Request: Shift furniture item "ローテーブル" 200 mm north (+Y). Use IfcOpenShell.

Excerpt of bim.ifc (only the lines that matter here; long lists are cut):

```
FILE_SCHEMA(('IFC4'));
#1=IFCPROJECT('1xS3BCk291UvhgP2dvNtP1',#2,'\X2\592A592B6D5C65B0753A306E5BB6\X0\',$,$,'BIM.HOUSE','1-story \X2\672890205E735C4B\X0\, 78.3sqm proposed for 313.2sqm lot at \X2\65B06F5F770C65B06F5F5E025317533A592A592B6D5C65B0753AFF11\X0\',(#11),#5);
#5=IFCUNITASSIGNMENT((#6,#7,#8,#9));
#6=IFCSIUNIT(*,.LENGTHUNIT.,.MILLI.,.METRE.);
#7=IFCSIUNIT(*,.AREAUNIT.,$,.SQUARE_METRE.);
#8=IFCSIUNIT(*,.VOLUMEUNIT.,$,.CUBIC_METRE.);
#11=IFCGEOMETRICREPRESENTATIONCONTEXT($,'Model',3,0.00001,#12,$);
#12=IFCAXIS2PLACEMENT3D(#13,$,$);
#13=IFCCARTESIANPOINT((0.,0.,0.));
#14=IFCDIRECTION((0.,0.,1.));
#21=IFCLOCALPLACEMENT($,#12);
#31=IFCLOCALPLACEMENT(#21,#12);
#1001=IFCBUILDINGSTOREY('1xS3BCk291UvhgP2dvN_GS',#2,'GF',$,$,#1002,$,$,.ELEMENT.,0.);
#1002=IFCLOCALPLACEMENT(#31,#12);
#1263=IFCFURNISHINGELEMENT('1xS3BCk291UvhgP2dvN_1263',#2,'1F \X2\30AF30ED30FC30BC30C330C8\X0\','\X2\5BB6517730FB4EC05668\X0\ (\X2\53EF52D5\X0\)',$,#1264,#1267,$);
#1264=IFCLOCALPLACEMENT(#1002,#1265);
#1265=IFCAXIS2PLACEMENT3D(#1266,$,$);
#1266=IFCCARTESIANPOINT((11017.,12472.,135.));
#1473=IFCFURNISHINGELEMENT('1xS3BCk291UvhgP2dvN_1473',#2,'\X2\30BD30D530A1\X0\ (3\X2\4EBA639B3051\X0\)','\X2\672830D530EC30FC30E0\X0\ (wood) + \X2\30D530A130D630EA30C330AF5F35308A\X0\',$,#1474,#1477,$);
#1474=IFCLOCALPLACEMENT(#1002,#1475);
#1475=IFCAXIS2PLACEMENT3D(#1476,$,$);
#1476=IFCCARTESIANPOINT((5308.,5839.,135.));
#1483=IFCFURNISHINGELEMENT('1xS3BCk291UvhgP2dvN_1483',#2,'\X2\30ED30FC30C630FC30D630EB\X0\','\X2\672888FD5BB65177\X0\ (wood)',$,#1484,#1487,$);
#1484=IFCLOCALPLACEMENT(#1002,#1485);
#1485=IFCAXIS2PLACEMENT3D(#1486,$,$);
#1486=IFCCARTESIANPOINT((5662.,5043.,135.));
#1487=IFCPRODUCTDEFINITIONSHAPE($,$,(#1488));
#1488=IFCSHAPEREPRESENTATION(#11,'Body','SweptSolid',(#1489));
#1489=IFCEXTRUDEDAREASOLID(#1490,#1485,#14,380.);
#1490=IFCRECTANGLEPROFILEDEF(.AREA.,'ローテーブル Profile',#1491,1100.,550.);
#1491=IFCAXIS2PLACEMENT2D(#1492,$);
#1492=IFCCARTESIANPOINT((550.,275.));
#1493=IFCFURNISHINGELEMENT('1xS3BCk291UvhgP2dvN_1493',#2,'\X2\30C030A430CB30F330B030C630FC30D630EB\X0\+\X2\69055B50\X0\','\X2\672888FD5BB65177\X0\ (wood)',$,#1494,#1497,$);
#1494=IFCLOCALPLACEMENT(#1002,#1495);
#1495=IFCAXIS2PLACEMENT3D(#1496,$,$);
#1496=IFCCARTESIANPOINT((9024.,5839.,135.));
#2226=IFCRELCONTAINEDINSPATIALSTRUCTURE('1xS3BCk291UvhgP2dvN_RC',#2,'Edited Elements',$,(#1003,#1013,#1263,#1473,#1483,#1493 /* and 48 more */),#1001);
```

```python
import ifcopenshell
import ifcopenshell.api.geometry
import ifcopenshell.util.placement
import ifcopenshell.util.unit

model = ifcopenshell.open("bim.ifc")
unit_scale = ifcopenshell.util.unit.calculate_unit_scale(model)

item = model.by_guid("1xS3BCk291UvhgP2dvN_1483")
matrix = ifcopenshell.util.placement.get_local_placement(item.ObjectPlacement)
matrix[1, 3] += 0.2 / unit_scale
ifcopenshell.api.geometry.edit_object_placement(model, product=item, matrix=matrix, is_si=False)

print(ifcopenshell.util.placement.get_local_placement(item.ObjectPlacement).round(3) + 0.0)

model.write("bim_edited.ifc")
```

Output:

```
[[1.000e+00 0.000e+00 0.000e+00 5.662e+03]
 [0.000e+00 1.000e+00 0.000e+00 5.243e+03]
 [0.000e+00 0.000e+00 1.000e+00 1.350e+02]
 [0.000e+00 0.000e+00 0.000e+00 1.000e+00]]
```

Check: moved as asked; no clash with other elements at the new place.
